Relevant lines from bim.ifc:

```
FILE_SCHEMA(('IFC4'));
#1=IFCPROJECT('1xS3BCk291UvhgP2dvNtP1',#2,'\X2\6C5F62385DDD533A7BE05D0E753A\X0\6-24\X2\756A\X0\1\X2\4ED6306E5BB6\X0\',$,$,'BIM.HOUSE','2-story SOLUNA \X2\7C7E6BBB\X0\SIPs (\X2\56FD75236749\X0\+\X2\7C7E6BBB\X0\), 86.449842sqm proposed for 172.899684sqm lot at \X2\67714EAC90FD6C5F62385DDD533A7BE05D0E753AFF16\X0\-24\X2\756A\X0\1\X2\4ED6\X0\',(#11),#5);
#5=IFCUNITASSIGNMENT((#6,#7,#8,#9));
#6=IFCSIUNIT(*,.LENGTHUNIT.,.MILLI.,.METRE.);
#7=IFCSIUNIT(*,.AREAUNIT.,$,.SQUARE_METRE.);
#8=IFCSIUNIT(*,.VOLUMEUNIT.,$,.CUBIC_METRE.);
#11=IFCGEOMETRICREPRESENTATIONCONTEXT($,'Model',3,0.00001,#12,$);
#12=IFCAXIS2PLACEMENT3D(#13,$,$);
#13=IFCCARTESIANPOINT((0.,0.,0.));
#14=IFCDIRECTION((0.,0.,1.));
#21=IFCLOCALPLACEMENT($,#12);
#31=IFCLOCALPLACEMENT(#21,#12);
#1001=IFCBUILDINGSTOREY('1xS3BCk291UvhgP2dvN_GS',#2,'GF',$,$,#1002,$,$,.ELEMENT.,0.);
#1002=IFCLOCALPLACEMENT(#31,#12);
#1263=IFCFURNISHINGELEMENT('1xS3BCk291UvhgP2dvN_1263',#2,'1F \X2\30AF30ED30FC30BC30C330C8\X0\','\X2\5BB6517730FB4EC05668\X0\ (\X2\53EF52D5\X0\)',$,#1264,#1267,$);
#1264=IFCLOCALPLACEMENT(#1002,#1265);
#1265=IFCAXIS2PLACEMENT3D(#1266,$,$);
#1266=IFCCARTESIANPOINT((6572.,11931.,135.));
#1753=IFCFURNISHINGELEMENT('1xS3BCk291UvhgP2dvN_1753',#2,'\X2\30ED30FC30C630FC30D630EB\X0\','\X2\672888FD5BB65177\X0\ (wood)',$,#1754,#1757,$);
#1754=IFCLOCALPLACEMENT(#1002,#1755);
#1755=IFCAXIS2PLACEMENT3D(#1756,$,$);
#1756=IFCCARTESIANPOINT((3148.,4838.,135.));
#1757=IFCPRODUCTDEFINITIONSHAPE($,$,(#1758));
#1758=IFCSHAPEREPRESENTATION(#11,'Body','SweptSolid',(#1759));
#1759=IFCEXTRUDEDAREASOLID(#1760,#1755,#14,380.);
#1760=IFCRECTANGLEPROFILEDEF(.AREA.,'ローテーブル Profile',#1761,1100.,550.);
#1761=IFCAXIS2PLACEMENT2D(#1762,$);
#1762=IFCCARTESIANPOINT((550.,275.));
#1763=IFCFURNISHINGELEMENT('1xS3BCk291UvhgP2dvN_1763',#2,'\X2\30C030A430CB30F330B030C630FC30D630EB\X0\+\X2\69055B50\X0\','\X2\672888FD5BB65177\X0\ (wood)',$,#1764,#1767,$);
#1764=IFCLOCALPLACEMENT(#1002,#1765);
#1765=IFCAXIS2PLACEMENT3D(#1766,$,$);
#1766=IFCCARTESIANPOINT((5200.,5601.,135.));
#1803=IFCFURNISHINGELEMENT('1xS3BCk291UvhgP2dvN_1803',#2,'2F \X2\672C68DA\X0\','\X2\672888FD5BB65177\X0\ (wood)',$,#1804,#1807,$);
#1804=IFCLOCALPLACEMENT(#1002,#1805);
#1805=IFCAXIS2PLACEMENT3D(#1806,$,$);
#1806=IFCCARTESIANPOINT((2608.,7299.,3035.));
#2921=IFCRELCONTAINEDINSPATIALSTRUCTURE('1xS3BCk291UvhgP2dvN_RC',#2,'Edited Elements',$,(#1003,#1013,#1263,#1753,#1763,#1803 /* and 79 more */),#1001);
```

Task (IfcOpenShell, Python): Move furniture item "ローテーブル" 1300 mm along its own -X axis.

```python
import ifcopenshell
import ifcopenshell.api.geometry
import ifcopenshell.util.placement
import ifcopenshell.util.unit

model = ifcopenshell.open("bim.ifc")
unit_scale = ifcopenshell.util.unit.calculate_unit_scale(model)

item = model.by_guid("1xS3BCk291UvhgP2dvN_1753")
matrix = ifcopenshell.util.placement.get_local_placement(item.ObjectPlacement)
matrix[:3, 3] -= matrix[:3, 0] * 1.3 / unit_scale
ifcopenshell.api.geometry.edit_object_placement(model, product=item, matrix=matrix, is_si=False)

print(ifcopenshell.util.placement.get_local_placement(item.ObjectPlacement).round(3) + 0.0)

model.write("bim_updated.ifc")
```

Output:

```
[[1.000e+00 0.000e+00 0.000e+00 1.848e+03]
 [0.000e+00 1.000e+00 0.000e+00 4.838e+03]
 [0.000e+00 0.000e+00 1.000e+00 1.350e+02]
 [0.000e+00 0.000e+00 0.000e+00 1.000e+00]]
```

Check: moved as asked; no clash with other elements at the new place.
